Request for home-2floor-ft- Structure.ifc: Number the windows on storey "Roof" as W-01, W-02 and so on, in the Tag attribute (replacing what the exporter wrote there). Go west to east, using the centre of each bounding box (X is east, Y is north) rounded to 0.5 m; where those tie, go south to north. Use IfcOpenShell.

First a look at what the model holds.

```python
import ifcopenshell
import ifcopenshell.util.element
import ifcopenshell.util.placement

model = ifcopenshell.open("home-2floor-ft- Structure.ifc")
print(model.schema)
storey = next(s for s in model.by_type("IfcBuildingStorey") if s.Name == "Roof")
windows = [e for e in ifcopenshell.util.element.get_decomposition(storey) if e.is_a("IfcWindow")]
for e in sorted(windows, key=lambda e: e.id()):
    origin = ifcopenshell.util.placement.get_local_placement(e.ObjectPlacement)[:3, 3]
    print(e.id(), e.Tag, e.Name, origin.round(2) + 0.0, sep=" | ")
```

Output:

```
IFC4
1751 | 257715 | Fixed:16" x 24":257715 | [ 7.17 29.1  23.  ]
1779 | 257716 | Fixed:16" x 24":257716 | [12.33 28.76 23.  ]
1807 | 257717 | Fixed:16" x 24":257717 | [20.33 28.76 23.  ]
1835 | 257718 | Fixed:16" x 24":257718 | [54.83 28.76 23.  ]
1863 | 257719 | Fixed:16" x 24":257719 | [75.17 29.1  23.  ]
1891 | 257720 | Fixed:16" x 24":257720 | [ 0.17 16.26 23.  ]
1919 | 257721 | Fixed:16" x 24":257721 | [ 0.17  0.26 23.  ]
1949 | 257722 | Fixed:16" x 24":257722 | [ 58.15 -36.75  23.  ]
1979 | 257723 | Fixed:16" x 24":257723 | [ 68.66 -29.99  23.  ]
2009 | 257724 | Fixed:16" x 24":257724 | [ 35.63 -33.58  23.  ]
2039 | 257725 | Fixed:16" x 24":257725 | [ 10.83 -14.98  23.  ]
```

```python
import ifcopenshell
import ifcopenshell.geom
import ifcopenshell.util.element
import ifcopenshell.util.shape

model = ifcopenshell.open("home-2floor-ft- Structure.ifc")
settings = ifcopenshell.geom.settings()
settings.set("use-world-coords", True)


def centre(element):
    shape = ifcopenshell.geom.create_shape(settings, element)
    return ifcopenshell.util.shape.get_bbox_centroid(shape.geometry)


storey = next(s for s in model.by_type("IfcBuildingStorey") if s.Name == "Roof")
windows = [e for e in ifcopenshell.util.element.get_decomposition(storey) if e.is_a("IfcWindow")]

# Insertion points can sit at a corner or the storey origin, so sort by the geometry (in metres).
centres = {e: centre(e) for e in windows}
windows.sort(key=lambda e: (round(centres[e][0] / 0.5), centres[e][1]))

for i, e in enumerate(windows, start=1):
    number = f"W-{i:02d}"
    e.Tag = number
    print(e.id(), number)

model.write("home-2floor-ft- Structure_v2.ifc")
```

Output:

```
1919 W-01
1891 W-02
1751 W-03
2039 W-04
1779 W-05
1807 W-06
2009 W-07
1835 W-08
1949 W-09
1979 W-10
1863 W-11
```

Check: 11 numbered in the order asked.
